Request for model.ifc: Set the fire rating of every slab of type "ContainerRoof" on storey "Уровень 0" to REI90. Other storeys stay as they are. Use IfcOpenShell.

First a look at what the model holds.

```python
import ifcopenshell
import ifcopenshell.util.element

model = ifcopenshell.open("model.ifc")
print(model.schema)
storey = next(s for s in model.by_type("IfcBuildingStorey") if s.Name == "Уровень 0")
slabs = [e for e in ifcopenshell.util.element.get_decomposition(storey) if e.is_a("IfcSlab")]
seen = {}
for e in slabs:
    element_type = ifcopenshell.util.element.get_type(e)
    key = (element_type.Name if element_type != e and element_type else None, ifcopenshell.util.element.get_pset(e, "Pset_SlabCommon", "FireRating"))
    seen[key] = seen.get(key, 0) + 1
for (name, value), count in sorted(seen.items(), key=str):
    print(count, "x", name, "|", value)
```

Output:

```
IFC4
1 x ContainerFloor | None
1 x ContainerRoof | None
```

```python
import ifcopenshell
import ifcopenshell.api.pset
import ifcopenshell.util.element

model = ifcopenshell.open("model.ifc")

storey = next(s for s in model.by_type("IfcBuildingStorey") if s.Name == "Уровень 0")
slabs = [e for e in ifcopenshell.util.element.get_decomposition(storey) if e.is_a("IfcSlab")]

count = 0
for e in slabs:
    element_type = ifcopenshell.util.element.get_type(e)
    if element_type in (None, e) or element_type.Name != "ContainerRoof":
        continue
    # add_pset returns the element's existing set when there is one.
    pset = ifcopenshell.api.pset.add_pset(model, product=e, name="Pset_SlabCommon")
    ifcopenshell.api.pset.edit_pset(model, pset=pset, properties={"FireRating": "REI90"})
    count += 1

print(count, "slabs updated")

model.write("model_rev.ifc")
```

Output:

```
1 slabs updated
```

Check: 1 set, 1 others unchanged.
